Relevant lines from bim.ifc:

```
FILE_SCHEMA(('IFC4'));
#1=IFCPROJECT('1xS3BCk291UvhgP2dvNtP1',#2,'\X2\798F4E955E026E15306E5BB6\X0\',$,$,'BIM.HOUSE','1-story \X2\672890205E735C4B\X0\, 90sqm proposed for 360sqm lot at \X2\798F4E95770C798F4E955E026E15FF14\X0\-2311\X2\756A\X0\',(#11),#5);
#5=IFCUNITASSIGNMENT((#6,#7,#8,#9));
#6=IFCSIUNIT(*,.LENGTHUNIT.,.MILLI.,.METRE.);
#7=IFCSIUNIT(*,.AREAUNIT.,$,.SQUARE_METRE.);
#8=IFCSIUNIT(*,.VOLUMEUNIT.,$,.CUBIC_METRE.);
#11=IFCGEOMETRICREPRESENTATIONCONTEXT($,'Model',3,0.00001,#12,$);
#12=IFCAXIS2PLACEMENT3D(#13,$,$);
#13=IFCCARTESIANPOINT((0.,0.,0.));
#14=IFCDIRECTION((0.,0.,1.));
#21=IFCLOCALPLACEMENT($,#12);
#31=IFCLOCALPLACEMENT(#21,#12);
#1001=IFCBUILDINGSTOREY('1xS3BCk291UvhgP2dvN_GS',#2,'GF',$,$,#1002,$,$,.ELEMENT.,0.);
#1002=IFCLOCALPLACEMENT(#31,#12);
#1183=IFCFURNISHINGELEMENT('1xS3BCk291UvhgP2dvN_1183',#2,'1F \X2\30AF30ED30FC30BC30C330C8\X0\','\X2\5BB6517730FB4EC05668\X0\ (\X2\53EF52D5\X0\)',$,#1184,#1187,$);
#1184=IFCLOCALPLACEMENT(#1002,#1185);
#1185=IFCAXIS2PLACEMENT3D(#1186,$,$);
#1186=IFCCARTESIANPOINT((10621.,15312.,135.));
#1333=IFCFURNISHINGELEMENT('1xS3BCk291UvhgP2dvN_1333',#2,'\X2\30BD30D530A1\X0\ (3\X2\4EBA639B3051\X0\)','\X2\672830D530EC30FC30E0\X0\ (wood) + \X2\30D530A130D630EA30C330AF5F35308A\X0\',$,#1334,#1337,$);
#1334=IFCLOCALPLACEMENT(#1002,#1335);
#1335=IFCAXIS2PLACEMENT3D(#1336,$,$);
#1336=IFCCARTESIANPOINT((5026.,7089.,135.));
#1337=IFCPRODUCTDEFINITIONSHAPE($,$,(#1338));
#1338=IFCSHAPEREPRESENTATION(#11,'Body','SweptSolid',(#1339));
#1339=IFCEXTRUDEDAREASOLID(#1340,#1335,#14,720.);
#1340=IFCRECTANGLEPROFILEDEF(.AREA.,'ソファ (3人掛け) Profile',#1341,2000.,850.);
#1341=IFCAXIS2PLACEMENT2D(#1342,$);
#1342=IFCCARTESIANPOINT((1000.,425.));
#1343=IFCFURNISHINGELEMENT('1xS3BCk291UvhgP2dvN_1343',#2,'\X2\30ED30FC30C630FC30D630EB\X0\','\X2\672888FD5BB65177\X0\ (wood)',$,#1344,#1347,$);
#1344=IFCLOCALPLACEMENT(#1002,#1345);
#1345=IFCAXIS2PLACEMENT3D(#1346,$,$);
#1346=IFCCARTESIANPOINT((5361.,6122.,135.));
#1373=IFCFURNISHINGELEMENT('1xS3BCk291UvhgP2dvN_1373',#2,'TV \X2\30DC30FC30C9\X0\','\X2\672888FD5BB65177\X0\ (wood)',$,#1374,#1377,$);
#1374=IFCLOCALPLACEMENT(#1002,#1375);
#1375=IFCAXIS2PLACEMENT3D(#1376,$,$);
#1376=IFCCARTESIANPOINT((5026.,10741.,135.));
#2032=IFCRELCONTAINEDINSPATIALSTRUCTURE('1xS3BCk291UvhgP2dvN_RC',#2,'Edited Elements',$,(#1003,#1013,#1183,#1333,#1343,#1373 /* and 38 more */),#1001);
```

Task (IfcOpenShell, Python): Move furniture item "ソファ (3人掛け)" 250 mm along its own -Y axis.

```python
import ifcopenshell
import ifcopenshell.api.geometry
import ifcopenshell.util.placement
import ifcopenshell.util.unit

model = ifcopenshell.open("bim.ifc")
unit_scale = ifcopenshell.util.unit.calculate_unit_scale(model)

item = model.by_guid("1xS3BCk291UvhgP2dvN_1333")
matrix = ifcopenshell.util.placement.get_local_placement(item.ObjectPlacement)
matrix[:3, 3] -= matrix[:3, 1] * 0.25 / unit_scale
ifcopenshell.api.geometry.edit_object_placement(model, product=item, matrix=matrix, is_si=False)

print(ifcopenshell.util.placement.get_local_placement(item.ObjectPlacement).round(3) + 0.0)

model.write("bim_updated.ifc")
```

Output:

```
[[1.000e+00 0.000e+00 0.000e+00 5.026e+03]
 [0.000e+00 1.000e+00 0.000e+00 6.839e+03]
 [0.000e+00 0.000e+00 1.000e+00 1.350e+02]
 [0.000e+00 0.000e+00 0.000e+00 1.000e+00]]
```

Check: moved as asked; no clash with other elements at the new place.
